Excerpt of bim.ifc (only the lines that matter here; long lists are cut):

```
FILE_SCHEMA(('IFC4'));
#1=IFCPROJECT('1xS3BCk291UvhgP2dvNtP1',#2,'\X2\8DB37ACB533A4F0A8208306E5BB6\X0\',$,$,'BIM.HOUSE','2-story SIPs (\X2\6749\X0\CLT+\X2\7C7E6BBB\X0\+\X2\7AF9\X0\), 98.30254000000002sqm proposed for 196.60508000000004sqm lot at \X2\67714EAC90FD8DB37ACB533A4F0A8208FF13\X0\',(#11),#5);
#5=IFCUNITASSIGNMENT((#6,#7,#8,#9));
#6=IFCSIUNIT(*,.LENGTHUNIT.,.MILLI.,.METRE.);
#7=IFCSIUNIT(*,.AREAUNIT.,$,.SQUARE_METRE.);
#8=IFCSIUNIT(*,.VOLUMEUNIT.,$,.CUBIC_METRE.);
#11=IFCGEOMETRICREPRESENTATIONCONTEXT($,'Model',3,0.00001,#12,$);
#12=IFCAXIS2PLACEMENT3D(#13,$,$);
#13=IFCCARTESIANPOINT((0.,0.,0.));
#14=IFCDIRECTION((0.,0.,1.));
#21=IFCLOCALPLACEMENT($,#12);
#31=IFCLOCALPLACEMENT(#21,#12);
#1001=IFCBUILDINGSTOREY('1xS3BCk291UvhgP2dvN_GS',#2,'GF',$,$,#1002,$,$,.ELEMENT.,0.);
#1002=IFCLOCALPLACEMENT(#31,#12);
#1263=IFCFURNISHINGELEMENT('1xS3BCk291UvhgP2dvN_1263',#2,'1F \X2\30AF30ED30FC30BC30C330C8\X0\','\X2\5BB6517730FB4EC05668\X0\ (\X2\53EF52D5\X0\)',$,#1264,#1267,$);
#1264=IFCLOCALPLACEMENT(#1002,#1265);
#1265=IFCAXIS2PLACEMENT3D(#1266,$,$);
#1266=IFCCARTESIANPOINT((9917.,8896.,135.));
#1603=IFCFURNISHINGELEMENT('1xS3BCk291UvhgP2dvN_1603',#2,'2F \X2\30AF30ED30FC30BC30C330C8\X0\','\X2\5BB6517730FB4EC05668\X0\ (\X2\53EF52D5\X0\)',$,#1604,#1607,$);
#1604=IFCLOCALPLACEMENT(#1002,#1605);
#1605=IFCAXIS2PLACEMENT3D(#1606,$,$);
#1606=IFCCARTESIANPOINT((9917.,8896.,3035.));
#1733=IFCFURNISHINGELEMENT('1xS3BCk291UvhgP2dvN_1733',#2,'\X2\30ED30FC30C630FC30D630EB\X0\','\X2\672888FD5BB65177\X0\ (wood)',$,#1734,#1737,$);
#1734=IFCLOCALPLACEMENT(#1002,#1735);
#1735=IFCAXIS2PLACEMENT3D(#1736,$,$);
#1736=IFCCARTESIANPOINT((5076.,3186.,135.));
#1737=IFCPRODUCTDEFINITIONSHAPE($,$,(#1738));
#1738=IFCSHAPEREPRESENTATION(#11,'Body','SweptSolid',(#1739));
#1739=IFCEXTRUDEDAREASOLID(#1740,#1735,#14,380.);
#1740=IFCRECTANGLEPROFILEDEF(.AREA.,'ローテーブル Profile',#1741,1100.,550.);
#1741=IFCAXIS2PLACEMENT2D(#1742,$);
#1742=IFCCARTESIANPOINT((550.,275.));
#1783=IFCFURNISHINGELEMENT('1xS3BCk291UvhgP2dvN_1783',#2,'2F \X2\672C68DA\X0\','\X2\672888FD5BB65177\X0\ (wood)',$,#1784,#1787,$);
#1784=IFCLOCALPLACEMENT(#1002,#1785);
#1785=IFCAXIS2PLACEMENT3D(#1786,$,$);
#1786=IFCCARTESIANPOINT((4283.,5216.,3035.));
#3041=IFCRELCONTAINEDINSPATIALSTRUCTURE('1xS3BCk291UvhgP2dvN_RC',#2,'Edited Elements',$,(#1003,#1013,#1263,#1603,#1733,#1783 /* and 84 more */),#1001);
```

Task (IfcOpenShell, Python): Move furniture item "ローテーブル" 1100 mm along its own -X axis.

```python
import ifcopenshell
import ifcopenshell.api.geometry
import ifcopenshell.util.placement
import ifcopenshell.util.unit

model = ifcopenshell.open("bim.ifc")
unit_scale = ifcopenshell.util.unit.calculate_unit_scale(model)

item = model.by_guid("1xS3BCk291UvhgP2dvN_1733")
matrix = ifcopenshell.util.placement.get_local_placement(item.ObjectPlacement)
matrix[:3, 3] -= matrix[:3, 0] * 1.1 / unit_scale
ifcopenshell.api.geometry.edit_object_placement(model, product=item, matrix=matrix, is_si=False)

print(ifcopenshell.util.placement.get_local_placement(item.ObjectPlacement).round(3) + 0.0)

model.write("bim_updated.ifc")
```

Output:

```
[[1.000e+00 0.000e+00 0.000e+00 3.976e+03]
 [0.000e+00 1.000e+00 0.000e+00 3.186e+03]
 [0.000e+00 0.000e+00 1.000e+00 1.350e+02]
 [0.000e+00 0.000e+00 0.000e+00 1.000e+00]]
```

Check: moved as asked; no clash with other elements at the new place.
